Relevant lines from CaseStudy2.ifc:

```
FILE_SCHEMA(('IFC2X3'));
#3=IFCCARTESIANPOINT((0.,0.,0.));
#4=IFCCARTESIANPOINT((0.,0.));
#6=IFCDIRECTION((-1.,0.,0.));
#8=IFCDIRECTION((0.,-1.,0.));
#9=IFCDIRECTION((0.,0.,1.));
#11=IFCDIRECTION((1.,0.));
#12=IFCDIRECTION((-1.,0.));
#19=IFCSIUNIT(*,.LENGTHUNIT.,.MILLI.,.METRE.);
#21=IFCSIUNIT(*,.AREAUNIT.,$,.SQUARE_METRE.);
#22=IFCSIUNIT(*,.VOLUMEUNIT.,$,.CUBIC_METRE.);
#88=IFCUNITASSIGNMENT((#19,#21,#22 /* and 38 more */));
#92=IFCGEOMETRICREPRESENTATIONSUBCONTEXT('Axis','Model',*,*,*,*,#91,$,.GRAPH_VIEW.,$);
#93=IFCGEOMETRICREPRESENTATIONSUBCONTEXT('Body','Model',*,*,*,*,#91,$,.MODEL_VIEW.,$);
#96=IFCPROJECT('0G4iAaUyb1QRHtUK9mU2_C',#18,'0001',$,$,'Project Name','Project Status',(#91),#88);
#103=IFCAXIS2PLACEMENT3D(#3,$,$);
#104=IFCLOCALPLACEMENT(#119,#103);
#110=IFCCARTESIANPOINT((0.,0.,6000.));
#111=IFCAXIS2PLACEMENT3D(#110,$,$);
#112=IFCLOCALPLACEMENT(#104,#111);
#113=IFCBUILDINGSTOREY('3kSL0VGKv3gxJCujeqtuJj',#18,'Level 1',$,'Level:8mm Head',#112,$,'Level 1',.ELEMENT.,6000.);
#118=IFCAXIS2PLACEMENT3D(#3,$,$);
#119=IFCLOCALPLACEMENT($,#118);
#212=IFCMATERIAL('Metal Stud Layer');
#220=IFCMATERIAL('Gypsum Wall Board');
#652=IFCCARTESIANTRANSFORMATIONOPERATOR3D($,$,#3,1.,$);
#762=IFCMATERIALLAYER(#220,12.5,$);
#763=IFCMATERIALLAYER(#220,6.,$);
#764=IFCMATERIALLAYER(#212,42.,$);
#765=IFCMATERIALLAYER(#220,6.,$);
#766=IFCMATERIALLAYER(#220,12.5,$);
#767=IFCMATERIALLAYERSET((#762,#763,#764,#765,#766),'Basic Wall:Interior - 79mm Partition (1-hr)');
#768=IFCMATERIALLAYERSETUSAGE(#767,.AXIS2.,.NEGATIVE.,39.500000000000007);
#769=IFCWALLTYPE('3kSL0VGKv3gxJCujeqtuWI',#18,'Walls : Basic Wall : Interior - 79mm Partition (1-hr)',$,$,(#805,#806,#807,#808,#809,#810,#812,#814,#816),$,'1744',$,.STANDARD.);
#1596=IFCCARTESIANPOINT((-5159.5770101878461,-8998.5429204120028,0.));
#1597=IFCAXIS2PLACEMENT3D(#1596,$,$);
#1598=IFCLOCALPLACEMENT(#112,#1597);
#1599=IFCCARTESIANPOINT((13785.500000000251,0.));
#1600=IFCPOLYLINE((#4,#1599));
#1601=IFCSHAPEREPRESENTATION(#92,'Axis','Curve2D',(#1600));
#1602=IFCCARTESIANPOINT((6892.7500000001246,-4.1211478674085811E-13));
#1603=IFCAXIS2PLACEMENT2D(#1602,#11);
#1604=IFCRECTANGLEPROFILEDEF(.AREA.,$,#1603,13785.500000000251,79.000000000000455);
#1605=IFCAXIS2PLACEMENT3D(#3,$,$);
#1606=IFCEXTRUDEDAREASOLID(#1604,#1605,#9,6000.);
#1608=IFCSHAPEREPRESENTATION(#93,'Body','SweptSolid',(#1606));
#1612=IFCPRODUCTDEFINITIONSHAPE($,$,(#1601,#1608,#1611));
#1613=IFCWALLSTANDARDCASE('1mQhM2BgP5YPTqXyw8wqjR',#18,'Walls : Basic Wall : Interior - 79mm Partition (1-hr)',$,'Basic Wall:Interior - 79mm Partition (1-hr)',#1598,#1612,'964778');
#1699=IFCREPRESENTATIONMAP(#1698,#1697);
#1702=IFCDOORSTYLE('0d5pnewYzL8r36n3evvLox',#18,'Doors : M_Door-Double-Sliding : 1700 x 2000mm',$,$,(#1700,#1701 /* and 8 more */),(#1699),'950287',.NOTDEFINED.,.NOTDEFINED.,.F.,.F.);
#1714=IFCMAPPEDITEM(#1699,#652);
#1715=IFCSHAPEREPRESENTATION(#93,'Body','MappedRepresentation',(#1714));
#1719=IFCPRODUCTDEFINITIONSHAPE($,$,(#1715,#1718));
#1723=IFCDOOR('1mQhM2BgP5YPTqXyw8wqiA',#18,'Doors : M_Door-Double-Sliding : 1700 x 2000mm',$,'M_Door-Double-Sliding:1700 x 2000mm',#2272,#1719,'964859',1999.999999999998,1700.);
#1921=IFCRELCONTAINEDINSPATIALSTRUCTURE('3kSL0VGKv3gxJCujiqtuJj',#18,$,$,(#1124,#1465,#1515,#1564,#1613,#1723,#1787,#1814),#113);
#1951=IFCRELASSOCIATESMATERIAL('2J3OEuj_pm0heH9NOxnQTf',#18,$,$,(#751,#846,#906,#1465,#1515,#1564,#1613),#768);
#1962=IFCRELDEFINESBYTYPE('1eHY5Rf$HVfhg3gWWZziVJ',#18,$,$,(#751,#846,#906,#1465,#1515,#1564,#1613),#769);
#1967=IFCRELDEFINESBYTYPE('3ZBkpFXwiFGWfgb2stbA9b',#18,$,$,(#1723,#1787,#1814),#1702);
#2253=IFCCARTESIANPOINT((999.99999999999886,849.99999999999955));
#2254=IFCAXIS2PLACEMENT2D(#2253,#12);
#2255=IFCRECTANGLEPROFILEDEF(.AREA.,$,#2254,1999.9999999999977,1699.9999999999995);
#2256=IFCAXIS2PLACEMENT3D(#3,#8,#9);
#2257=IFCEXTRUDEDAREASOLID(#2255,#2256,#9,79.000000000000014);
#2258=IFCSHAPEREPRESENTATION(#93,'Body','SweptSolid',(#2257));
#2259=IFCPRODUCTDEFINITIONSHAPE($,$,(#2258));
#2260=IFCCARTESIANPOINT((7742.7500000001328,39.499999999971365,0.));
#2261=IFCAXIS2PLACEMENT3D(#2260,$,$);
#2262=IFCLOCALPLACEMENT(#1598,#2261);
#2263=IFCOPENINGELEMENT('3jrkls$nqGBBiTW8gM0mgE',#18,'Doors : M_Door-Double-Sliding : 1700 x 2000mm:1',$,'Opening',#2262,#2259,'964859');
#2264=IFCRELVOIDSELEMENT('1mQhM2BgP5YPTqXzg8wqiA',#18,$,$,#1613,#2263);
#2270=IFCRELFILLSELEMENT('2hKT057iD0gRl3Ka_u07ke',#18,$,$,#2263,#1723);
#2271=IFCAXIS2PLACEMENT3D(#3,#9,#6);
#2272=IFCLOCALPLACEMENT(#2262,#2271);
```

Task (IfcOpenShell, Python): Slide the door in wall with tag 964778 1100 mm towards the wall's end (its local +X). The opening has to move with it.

```python
import ifcopenshell
import ifcopenshell.api.geometry
import ifcopenshell.util.placement

model = ifcopenshell.open("CaseStudy2.ifc")

door = model.by_id(1723)
opening = door.FillsVoids[0].RelatingOpeningElement
wall = opening.VoidsElements[0].RelatingBuildingElement

wall_matrix = ifcopenshell.util.placement.get_local_placement(wall.ObjectPlacement)
shift = wall_matrix[:3, 0] * 1100.0
before = ifcopenshell.util.placement.get_local_placement(door.ObjectPlacement)[:3, 3].copy()

# The door is placed relative to its opening, so it follows when the opening moves.
matrix = ifcopenshell.util.placement.get_local_placement(opening.ObjectPlacement)
matrix[:3, 3] += shift
ifcopenshell.api.geometry.edit_object_placement(
    model, product=opening, matrix=matrix, is_si=False, should_transform_children=True
)

after = ifcopenshell.util.placement.get_local_placement(door.ObjectPlacement)[:3, 3]
print("door moved by", (after - before).round(3) + 0.0)

model.write("CaseStudy2-out.ifc")
```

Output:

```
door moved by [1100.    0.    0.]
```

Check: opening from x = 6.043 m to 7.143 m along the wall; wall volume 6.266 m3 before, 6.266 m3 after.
